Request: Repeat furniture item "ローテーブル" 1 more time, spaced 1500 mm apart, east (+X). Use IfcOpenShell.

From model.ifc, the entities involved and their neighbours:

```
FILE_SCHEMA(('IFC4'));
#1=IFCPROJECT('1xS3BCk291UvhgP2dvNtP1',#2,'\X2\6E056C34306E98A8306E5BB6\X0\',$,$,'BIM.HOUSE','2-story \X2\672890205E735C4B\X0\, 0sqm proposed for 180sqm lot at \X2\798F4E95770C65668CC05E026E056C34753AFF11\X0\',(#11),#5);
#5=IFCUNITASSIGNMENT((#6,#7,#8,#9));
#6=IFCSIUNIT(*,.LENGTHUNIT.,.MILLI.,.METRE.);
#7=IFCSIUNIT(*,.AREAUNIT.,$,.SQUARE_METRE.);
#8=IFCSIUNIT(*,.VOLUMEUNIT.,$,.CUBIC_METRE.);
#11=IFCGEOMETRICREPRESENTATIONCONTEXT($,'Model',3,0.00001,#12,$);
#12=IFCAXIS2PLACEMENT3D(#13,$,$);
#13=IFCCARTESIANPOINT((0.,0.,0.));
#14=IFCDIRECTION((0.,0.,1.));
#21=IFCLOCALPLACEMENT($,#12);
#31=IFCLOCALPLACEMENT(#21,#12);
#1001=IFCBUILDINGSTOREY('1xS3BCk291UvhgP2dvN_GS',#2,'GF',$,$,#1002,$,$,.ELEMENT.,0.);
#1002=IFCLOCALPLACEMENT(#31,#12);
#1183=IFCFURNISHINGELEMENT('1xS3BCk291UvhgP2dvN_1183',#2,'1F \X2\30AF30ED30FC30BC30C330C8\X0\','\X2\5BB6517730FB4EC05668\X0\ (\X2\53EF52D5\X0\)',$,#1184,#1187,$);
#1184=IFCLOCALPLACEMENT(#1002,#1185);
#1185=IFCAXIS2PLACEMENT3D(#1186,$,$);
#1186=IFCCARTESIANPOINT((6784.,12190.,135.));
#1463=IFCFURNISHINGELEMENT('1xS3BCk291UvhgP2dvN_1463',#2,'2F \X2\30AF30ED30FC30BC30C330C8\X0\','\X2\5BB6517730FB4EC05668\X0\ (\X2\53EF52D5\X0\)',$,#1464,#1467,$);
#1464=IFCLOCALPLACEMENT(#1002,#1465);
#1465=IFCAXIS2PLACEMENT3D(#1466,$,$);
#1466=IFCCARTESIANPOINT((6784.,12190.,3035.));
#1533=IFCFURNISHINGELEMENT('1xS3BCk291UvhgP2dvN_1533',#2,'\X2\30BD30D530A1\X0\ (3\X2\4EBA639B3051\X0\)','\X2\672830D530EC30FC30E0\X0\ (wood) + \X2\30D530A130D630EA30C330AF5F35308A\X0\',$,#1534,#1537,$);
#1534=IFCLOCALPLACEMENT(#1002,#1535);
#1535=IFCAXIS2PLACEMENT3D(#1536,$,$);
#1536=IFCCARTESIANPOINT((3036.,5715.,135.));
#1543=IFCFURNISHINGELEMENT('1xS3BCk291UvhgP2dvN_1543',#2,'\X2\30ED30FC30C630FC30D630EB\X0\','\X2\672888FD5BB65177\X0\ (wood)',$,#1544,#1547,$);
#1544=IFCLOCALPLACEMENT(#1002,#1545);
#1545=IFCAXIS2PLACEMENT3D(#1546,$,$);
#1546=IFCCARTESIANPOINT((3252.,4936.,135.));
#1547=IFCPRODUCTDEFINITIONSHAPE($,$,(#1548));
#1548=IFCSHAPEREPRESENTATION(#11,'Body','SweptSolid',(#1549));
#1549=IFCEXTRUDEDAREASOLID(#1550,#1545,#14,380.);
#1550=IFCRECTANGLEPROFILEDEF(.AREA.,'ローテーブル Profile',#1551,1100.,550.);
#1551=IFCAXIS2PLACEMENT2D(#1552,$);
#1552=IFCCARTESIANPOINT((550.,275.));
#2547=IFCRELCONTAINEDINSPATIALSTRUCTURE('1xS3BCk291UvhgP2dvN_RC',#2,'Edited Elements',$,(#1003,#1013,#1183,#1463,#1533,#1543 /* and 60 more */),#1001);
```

```python
import numpy as np
import ifcopenshell
import ifcopenshell.api.geometry
import ifcopenshell.api.root
import ifcopenshell.util.element
import ifcopenshell.util.placement

model = ifcopenshell.open("model.ifc")


def reuse_history(source, copy):
    """copy_class also copies each property set's owner history, people and application; keep the originals."""
    for rel in copy.IsDefinedBy:
        if rel.is_a("IfcRelDefinesByProperties") and (history := rel.RelatingPropertyDefinition.OwnerHistory):
            rel.RelatingPropertyDefinition.OwnerHistory = source.OwnerHistory
            ifcopenshell.util.element.remove_deep2(model, history)


source = model.by_guid("1xS3BCk291UvhgP2dvN_1543")
base = ifcopenshell.util.placement.get_local_placement(source.ObjectPlacement)
step = np.array([1.0, 0.0, 0.0]) * 1500.0

for i in range(1, 2):
    copy = ifcopenshell.api.root.copy_class(model, product=source)
    copy.Representation = ifcopenshell.util.element.copy_deep(
        model, source.Representation, exclude=["IfcGeometricRepresentationContext", "IfcRepresentationMap"]
    )
    reuse_history(source, copy)
    matrix = base.copy()
    matrix[:3, 3] += i * step
    print("added at", matrix[:3, 3].round(3) + 0.0)
    ifcopenshell.api.geometry.edit_object_placement(model, product=copy, matrix=matrix, is_si=False)

model.write("model_edited.ifc")
```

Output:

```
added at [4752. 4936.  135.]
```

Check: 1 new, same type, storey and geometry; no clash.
